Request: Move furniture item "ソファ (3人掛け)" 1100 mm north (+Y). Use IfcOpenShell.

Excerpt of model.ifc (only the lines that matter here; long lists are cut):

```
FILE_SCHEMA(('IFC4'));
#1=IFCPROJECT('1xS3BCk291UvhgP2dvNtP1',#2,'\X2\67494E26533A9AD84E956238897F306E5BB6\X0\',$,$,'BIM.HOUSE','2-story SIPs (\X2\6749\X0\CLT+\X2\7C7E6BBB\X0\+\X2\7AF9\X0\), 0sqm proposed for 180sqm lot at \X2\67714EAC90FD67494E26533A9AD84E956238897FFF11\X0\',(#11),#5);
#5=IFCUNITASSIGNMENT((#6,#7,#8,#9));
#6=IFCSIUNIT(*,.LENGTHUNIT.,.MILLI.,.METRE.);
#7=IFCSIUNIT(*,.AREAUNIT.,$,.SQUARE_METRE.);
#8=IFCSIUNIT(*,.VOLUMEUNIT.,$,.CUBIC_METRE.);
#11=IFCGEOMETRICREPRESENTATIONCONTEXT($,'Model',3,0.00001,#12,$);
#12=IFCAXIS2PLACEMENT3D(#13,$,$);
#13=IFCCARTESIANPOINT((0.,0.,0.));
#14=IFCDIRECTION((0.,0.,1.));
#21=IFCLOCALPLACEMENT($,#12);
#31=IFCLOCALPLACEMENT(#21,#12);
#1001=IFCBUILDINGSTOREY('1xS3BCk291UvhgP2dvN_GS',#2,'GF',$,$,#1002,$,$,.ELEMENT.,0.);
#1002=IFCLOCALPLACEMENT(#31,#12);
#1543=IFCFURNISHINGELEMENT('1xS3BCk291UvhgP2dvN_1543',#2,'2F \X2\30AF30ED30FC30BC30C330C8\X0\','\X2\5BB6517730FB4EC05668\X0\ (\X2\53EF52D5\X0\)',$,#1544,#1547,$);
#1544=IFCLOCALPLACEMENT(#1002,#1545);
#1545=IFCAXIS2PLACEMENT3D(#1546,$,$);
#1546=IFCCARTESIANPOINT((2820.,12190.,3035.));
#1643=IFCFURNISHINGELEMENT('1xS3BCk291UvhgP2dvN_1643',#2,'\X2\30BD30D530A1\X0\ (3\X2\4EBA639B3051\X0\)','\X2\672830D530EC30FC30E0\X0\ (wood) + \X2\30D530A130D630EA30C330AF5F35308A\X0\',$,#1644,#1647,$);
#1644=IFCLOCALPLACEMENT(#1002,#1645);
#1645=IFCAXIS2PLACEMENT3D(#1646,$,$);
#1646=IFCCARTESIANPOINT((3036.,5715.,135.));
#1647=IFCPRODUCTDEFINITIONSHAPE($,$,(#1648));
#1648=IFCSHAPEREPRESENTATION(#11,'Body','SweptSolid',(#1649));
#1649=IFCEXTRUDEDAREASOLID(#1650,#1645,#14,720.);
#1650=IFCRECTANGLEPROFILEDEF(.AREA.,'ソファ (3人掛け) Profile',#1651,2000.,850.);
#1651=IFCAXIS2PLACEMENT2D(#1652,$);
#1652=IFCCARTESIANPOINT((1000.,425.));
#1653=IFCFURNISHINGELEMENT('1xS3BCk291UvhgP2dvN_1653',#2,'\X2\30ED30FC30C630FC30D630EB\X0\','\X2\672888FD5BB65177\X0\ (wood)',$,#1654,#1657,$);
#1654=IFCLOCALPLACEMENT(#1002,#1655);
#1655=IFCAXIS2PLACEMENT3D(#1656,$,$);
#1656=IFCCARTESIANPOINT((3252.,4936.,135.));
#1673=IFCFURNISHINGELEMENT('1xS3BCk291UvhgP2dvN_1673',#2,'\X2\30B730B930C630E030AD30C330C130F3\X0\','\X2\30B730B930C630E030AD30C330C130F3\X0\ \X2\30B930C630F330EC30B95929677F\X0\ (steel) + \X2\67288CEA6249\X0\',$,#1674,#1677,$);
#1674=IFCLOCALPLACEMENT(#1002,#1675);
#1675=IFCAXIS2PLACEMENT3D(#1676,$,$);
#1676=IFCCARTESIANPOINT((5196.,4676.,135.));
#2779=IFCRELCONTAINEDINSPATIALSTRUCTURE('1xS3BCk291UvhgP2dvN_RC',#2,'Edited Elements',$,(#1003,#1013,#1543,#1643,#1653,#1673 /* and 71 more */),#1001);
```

```python
import ifcopenshell
import ifcopenshell.api.geometry
import ifcopenshell.util.placement

model = ifcopenshell.open("model.ifc")

item = model.by_guid("1xS3BCk291UvhgP2dvN_1643")
matrix = ifcopenshell.util.placement.get_local_placement(item.ObjectPlacement)
matrix[1, 3] += 1100.0
ifcopenshell.api.geometry.edit_object_placement(model, product=item, matrix=matrix, is_si=False)

print(ifcopenshell.util.placement.get_local_placement(item.ObjectPlacement).round(3) + 0.0)

model.write("model_v2.ifc")
```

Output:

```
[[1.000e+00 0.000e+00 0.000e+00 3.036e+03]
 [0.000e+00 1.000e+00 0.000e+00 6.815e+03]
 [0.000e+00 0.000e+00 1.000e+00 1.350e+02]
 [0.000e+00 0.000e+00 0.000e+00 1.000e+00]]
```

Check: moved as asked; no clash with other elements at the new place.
